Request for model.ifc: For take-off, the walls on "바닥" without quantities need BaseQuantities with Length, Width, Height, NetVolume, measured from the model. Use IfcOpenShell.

First a look at what the model holds.

```python
import ifcopenshell
import ifcopenshell.util.element
import ifcopenshell.util.unit

model = ifcopenshell.open("model.ifc")
print(model.schema)
for unit_type in ("LENGTHUNIT", "AREAUNIT", "VOLUMEUNIT"):
    print(unit_type, ifcopenshell.util.unit.calculate_unit_scale(model, unit_type))
storey = next(s for s in model.by_type("IfcBuildingStorey") if s.Name == "바닥")
walls = [e for e in ifcopenshell.util.element.get_decomposition(storey) if e.is_a("IfcWall")]
for e in sorted(walls, key=lambda e: e.id()):
    print(e.id(), e.is_a(), e.Name, list(ifcopenshell.util.element.get_psets(e, qtos_only=True)), sep=" | ")
```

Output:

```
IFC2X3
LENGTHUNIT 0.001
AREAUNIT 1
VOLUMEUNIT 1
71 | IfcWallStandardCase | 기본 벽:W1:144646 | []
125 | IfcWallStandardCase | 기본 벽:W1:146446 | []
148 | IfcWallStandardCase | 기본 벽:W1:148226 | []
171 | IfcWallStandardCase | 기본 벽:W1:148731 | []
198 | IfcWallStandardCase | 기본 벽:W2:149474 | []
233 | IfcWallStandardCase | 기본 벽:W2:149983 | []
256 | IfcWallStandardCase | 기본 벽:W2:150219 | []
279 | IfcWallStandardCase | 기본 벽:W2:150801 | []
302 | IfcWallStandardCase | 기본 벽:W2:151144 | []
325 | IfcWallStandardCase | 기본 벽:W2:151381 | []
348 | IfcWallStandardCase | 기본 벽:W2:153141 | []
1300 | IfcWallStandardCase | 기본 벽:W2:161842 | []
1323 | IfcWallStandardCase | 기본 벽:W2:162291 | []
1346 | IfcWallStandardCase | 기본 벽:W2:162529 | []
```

```python
import ifcopenshell
import ifcopenshell.api.pset
import ifcopenshell.geom
import ifcopenshell.util.element
import ifcopenshell.util.shape
import ifcopenshell.util.unit

model = ifcopenshell.open("model.ifc")
unit_scale = ifcopenshell.util.unit.calculate_unit_scale(model)
volume_scale = ifcopenshell.util.unit.calculate_unit_scale(model, "VOLUMEUNIT")
settings = ifcopenshell.geom.settings()

storey = next(s for s in model.by_type("IfcBuildingStorey") if s.Name == "바닥")
walls = [e for e in ifcopenshell.util.element.get_decomposition(storey) if e.is_a("IfcWall")]

for e in sorted(walls, key=lambda e: e.id()):
    if ifcopenshell.util.element.get_psets(e, qtos_only=True, should_inherit=False):
        continue
    # Geometry comes back in metres, in the element's own axes.
    shape = ifcopenshell.geom.create_shape(settings, e)
    values = {
        "Length": ifcopenshell.util.shape.get_x(shape.geometry) / unit_scale,
        "Width": ifcopenshell.util.shape.get_y(shape.geometry) / unit_scale,
        "Height": ifcopenshell.util.shape.get_z(shape.geometry) / unit_scale,
        "NetVolume": ifcopenshell.util.shape.get_volume(shape.geometry) / volume_scale,
    }
    qto = ifcopenshell.api.pset.add_qto(model, product=e, name="BaseQuantities")
    ifcopenshell.api.pset.edit_qto(model, qto=qto, properties=values)
    print(e.id(), {k: round(v, 3) for k, v in values.items()})

model.write("model_rev.ifc")
```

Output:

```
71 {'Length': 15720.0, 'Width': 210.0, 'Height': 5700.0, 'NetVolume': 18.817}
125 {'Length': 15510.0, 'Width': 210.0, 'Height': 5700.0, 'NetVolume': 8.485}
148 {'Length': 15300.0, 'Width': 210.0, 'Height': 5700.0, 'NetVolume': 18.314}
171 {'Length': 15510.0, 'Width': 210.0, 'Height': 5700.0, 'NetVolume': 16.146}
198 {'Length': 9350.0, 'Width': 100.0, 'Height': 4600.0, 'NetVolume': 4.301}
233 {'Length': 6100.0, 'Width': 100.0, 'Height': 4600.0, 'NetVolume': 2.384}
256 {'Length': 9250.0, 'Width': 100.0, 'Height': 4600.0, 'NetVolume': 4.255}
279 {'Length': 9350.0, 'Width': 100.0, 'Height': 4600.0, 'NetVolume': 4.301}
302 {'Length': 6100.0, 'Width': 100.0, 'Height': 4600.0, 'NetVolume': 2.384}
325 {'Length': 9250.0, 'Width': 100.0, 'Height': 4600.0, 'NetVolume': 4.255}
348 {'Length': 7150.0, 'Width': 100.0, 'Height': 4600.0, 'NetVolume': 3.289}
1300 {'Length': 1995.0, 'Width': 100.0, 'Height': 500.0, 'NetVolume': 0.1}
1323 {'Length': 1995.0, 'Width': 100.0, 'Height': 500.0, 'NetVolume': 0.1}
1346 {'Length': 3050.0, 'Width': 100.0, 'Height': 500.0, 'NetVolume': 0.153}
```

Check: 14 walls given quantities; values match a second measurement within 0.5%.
